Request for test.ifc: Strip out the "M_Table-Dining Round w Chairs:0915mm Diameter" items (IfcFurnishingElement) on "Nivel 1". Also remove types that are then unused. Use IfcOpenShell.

First a look at what the model holds.

```python
import ifcopenshell
import ifcopenshell.util.element

model = ifcopenshell.open("test.ifc")
print(model.schema)
storey = next(s for s in model.by_type("IfcBuildingStorey") if s.Name == "Nivel 1")
furniture = [e for e in ifcopenshell.util.element.get_decomposition(storey) if e.is_a("IfcFurnishingElement")]
seen = {}
for e in furniture:
    element_type = ifcopenshell.util.element.get_type(e)
    name = element_type.Name if element_type not in (None, e) else None
    seen[name] = seen.get(name, 0) + 1
for name, count in sorted(seen.items(), key=str):
    print(count, "x", name)
```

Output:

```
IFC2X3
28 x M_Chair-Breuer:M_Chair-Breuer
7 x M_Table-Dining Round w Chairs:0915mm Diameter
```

```python
import ifcopenshell
import ifcopenshell.api.root
import ifcopenshell.util.element

model = ifcopenshell.open("test.ifc")

storey = next(s for s in model.by_type("IfcBuildingStorey") if s.Name == "Nivel 1")
furniture = [e for e in ifcopenshell.util.element.get_decomposition(storey) if e.is_a("IfcFurnishingElement")]
targets = [e for e in furniture if (t := ifcopenshell.util.element.get_type(e)) not in (None, e) and t.Name == "M_Table-Dining Round w Chairs:0915mm Diameter"]
types = {ifcopenshell.util.element.get_type(e) for e in targets} - {None, *targets}

for e in targets:
    ifcopenshell.api.root.remove_product(model, product=e)
print(len(targets), "removed")

unused = [t for t in types if not ifcopenshell.util.element.get_types(t)]
for t in unused:
    ifcopenshell.api.root.remove_product(model, product=t)
print(len(unused), "unused types removed")

model.write("test_edited.ifc")
```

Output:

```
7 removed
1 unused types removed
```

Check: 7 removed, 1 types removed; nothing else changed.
